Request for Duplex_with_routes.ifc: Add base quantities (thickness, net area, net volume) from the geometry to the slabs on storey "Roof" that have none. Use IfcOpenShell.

First a look at what the model holds.

```python
import ifcopenshell
import ifcopenshell.util.element
import ifcopenshell.util.unit

model = ifcopenshell.open("Duplex_with_routes.ifc")
print(model.schema)
for unit_type in ("LENGTHUNIT", "AREAUNIT", "VOLUMEUNIT"):
    print(unit_type, ifcopenshell.util.unit.calculate_unit_scale(model, unit_type))
storey = next(s for s in model.by_type("IfcBuildingStorey") if s.Name == "Roof")
slabs = [e for e in ifcopenshell.util.element.get_decomposition(storey) if e.is_a("IfcSlab")]
for e in sorted(slabs, key=lambda e: e.id()):
    print(e.id(), e.is_a(), e.Name, list(ifcopenshell.util.element.get_psets(e, qtos_only=True)), sep=" | ")
```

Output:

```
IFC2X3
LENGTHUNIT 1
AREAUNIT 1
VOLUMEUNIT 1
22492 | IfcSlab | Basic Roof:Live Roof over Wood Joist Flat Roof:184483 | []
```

```python
import ifcopenshell
import ifcopenshell.api.pset
import ifcopenshell.geom
import ifcopenshell.util.element
import ifcopenshell.util.shape
import ifcopenshell.util.unit

model = ifcopenshell.open("Duplex_with_routes.ifc")
unit_scale = ifcopenshell.util.unit.calculate_unit_scale(model)
area_scale = ifcopenshell.util.unit.calculate_unit_scale(model, "AREAUNIT")
volume_scale = ifcopenshell.util.unit.calculate_unit_scale(model, "VOLUMEUNIT")
settings = ifcopenshell.geom.settings()

storey = next(s for s in model.by_type("IfcBuildingStorey") if s.Name == "Roof")
slabs = [e for e in ifcopenshell.util.element.get_decomposition(storey) if e.is_a("IfcSlab")]

for e in sorted(slabs, key=lambda e: e.id()):
    if ifcopenshell.util.element.get_psets(e, qtos_only=True, should_inherit=False):
        continue
    # Geometry comes back in metres, in the element's own axes.
    shape = ifcopenshell.geom.create_shape(settings, e)
    values = {
        "Width": ifcopenshell.util.shape.get_z(shape.geometry) / unit_scale,
        "NetArea": ifcopenshell.util.shape.get_footprint_area(shape.geometry) / area_scale,
        "NetVolume": ifcopenshell.util.shape.get_volume(shape.geometry) / volume_scale,
    }
    qto = ifcopenshell.api.pset.add_qto(model, product=e, name="BaseQuantities")
    ifcopenshell.api.pset.edit_qto(model, qto=qto, properties=values)
    print(e.id(), {k: round(v, 3) for k, v in values.items()})

model.write("Duplex_with_routes_rev.ifc")
```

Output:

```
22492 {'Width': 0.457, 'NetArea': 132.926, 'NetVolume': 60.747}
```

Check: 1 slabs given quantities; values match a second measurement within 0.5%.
